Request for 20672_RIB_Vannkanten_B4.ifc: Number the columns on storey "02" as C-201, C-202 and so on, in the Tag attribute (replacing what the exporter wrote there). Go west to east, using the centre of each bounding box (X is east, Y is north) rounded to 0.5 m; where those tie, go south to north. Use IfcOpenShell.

First a look at what the model holds.

```python
import ifcopenshell
import ifcopenshell.util.element
import ifcopenshell.util.placement

model = ifcopenshell.open("20672_RIB_Vannkanten_B4.ifc")
print(model.schema)
storey = next(s for s in model.by_type("IfcBuildingStorey") if s.Name == "02")
columns = [e for e in ifcopenshell.util.element.get_decomposition(storey) if e.is_a("IfcColumn")]
for e in sorted(columns, key=lambda e: e.id()):
    origin = ifcopenshell.util.placement.get_local_placement(e.ObjectPlacement)[:3, 3]
    print(e.id(), e.Tag, e.Name, origin.round(2) + 0.0, sep=" | ")
```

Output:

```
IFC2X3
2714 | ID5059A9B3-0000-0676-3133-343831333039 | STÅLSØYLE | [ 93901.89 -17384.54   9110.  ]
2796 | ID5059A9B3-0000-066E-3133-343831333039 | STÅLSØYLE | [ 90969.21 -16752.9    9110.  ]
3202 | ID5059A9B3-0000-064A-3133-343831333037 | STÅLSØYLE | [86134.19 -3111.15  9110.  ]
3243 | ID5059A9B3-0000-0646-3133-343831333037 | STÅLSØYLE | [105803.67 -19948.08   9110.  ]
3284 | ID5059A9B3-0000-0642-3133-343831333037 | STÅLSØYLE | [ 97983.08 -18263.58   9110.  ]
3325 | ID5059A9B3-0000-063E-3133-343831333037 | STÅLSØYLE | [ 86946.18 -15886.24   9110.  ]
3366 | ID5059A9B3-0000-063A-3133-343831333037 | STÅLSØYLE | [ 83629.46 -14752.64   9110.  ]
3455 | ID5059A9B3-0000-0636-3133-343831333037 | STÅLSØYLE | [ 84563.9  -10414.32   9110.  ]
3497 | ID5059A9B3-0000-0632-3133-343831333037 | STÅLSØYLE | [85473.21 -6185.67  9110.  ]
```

```python
import ifcopenshell
import ifcopenshell.geom
import ifcopenshell.util.element
import ifcopenshell.util.shape

model = ifcopenshell.open("20672_RIB_Vannkanten_B4.ifc")
settings = ifcopenshell.geom.settings()
settings.set("use-world-coords", True)


def centre(element):
    shape = ifcopenshell.geom.create_shape(settings, element)
    return ifcopenshell.util.shape.get_bbox_centroid(shape.geometry)


storey = next(s for s in model.by_type("IfcBuildingStorey") if s.Name == "02")
columns = [e for e in ifcopenshell.util.element.get_decomposition(storey) if e.is_a("IfcColumn")]

# Insertion points can sit at a corner or the storey origin, so sort by the geometry (in metres).
centres = {e: centre(e) for e in columns}
columns.sort(key=lambda e: (round(centres[e][0] / 0.5), centres[e][1]))

for i, e in enumerate(columns, start=1):
    number = f"C-2{i:02d}"
    e.Tag = number
    print(e.id(), number)

model.write("20672_RIB_Vannkanten_B4_updated.ifc")
```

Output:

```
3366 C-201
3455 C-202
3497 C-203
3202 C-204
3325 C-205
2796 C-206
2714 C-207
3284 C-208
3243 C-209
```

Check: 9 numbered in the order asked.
